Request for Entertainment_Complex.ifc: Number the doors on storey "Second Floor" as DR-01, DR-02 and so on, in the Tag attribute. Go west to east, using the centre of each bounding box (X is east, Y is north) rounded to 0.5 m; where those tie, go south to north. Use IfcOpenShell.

First a look at what the model holds.

```python
import ifcopenshell
import ifcopenshell.util.element
import ifcopenshell.util.placement

model = ifcopenshell.open("Entertainment_Complex.ifc")
print(model.schema)
storey = next(s for s in model.by_type("IfcBuildingStorey") if s.Name == "Second Floor")
doors = [e for e in ifcopenshell.util.element.get_decomposition(storey) if e.is_a("IfcDoor")]
for e in sorted(doors, key=lambda e: e.id()):
    origin = ifcopenshell.util.placement.get_local_placement(e.ObjectPlacement)[:3, 3]
    print(e.id(), e.Tag, e.Name, origin.round(2) + 0.0, sep=" | ")
```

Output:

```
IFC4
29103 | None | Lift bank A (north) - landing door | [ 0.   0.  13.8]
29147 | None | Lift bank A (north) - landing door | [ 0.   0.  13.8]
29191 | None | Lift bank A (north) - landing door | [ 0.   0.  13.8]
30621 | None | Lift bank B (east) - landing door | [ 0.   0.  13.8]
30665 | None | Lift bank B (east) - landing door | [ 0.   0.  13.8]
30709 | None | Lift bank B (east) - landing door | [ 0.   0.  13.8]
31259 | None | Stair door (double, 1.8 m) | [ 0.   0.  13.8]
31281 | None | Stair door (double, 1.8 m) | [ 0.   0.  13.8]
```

```python
import ifcopenshell
import ifcopenshell.geom
import ifcopenshell.util.element
import ifcopenshell.util.shape

model = ifcopenshell.open("Entertainment_Complex.ifc")
settings = ifcopenshell.geom.settings()
settings.set("use-world-coords", True)


def centre(element):
    shape = ifcopenshell.geom.create_shape(settings, element)
    return ifcopenshell.util.shape.get_bbox_centroid(shape.geometry)


storey = next(s for s in model.by_type("IfcBuildingStorey") if s.Name == "Second Floor")
doors = [e for e in ifcopenshell.util.element.get_decomposition(storey) if e.is_a("IfcDoor")]

# Insertion points can sit at a corner or the storey origin, so sort by the geometry (in metres).
centres = {e: centre(e) for e in doors}
doors.sort(key=lambda e: (round(centres[e][0] / 0.5), centres[e][1]))

for i, e in enumerate(doors, start=1):
    number = f"DR-{i:02d}"
    e.Tag = number
    print(e.id(), number)

model.write("Entertainment_Complex-out.ifc")
```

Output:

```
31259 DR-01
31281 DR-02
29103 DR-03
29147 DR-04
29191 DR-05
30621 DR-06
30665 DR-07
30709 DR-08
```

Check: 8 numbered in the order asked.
